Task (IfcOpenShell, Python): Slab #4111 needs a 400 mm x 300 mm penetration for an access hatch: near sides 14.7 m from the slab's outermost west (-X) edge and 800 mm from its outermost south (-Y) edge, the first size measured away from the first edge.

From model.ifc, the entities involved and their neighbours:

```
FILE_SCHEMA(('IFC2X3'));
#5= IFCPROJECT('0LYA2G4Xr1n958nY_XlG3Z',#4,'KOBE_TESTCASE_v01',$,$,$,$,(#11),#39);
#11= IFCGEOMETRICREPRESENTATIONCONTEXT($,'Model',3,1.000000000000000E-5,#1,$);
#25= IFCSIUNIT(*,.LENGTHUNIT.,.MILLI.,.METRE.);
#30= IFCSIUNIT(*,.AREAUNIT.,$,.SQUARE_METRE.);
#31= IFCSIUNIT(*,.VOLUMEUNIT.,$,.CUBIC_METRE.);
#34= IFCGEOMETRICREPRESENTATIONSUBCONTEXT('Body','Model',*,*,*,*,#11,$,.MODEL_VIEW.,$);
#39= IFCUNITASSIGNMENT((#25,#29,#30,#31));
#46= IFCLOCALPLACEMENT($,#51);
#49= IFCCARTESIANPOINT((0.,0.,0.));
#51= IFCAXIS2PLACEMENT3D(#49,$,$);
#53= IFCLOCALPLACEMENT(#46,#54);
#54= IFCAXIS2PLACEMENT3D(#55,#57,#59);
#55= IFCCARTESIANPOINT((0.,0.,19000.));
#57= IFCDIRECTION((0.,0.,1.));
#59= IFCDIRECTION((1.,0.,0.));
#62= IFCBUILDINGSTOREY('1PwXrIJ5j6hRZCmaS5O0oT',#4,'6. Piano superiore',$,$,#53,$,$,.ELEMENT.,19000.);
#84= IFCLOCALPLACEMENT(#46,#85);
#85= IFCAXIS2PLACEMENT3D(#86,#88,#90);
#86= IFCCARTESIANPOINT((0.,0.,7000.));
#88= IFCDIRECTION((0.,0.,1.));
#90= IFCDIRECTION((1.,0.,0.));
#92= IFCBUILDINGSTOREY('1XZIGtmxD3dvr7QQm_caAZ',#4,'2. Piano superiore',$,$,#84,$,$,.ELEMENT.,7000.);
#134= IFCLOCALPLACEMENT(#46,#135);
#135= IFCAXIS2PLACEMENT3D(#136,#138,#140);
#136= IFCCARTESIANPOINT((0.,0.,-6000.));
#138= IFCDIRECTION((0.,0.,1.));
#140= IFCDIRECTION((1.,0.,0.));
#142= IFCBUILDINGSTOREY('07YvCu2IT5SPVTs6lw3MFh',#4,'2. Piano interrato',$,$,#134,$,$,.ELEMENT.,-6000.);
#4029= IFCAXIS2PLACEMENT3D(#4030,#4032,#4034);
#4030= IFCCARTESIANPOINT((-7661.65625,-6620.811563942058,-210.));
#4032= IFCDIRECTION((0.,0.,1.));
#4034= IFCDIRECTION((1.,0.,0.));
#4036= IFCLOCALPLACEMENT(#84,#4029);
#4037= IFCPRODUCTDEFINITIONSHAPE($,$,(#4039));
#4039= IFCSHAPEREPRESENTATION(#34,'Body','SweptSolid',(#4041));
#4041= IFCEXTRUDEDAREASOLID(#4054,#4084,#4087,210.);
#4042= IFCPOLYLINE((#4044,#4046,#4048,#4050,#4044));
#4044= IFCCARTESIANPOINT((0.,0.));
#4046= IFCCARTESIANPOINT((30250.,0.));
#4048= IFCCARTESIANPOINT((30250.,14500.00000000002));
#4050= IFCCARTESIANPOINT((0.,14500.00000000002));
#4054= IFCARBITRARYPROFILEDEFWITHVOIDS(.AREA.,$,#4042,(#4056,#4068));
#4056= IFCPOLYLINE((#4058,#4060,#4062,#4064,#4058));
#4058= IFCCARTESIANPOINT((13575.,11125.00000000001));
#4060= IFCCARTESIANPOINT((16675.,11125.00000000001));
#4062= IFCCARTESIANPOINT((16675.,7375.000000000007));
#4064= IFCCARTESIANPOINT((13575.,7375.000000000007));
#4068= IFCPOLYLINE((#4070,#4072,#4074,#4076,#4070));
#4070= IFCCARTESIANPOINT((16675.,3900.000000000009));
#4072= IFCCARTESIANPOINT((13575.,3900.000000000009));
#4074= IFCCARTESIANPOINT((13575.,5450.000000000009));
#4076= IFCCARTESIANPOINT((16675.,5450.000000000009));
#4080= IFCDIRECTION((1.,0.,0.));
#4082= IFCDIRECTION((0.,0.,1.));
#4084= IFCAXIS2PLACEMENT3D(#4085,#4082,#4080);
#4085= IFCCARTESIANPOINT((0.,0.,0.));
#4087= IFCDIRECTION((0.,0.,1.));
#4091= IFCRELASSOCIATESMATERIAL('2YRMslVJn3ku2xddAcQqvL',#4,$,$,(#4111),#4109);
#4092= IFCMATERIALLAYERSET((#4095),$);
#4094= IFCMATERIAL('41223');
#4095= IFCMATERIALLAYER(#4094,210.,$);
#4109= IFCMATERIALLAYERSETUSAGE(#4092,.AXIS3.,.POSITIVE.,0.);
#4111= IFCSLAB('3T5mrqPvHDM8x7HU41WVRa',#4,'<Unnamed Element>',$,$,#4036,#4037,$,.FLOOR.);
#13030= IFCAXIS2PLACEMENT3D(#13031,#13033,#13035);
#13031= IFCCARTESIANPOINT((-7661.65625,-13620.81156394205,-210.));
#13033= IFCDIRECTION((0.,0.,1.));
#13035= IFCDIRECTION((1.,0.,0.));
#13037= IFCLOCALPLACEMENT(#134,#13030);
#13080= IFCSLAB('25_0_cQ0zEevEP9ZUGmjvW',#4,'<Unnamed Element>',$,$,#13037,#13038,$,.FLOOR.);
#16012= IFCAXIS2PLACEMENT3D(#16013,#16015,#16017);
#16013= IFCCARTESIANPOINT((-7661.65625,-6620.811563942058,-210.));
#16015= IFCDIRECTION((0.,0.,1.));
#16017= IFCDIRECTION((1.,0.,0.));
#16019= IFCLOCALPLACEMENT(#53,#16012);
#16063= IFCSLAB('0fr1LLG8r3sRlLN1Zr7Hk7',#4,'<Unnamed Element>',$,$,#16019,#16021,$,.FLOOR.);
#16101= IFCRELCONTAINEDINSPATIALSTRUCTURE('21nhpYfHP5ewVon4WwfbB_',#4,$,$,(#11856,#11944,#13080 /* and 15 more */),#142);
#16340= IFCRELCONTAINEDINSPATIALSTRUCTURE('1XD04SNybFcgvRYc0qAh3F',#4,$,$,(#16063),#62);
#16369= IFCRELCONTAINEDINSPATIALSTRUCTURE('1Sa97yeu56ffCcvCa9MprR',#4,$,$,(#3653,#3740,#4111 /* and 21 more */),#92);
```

```python
import numpy as np
import ifcopenshell
import ifcopenshell.api.feature
import ifcopenshell.api.geometry
import ifcopenshell.api.root
import ifcopenshell.geom
import ifcopenshell.util.placement
import ifcopenshell.util.representation
import ifcopenshell.util.shape
import ifcopenshell.util.unit

model = ifcopenshell.open("model.ifc")
unit_scale = ifcopenshell.util.unit.calculate_unit_scale(model)
settings = ifcopenshell.geom.settings()


def volume(element):
    """Net volume in cubic metres, openings subtracted."""
    shape = ifcopenshell.geom.create_shape(settings, element)
    return ifcopenshell.util.shape.get_volume(shape.geometry)


slab = model.by_guid("3T5mrqPvHDM8x7HU41WVRa")
before = volume(slab)

# Extent in the slab's own axes, in metres. The edges named are its -X and -Y sides.
slab_shape = ifcopenshell.geom.create_shape(settings, slab)
vertices = ifcopenshell.util.shape.get_vertices(slab_shape.geometry)
x_min, y_min, bottom = vertices.min(axis=0)
top = vertices[:, 2].max()

opening = ifcopenshell.api.root.create_entity(model, ifc_class="IfcOpeningElement", name="Access hatch opening")
context = ifcopenshell.util.representation.get_context(model, "Model", "Body", "MODEL_VIEW")
width, depth = 0.4, 0.3
outline = [(0.0, 0.0), (width, 0.0), (width, depth), (0.0, depth), (0.0, 0.0)]
# Overshoot both faces by 50 mm so the cut is clean.
shape = ifcopenshell.api.geometry.add_slab_representation(
    model, context=context, depth=top - bottom + 0.1, polyline=outline
)
ifcopenshell.api.geometry.assign_representation(model, product=opening, representation=shape)

matrix = ifcopenshell.util.placement.get_local_placement(slab.ObjectPlacement)
matrix[:, 3] = matrix @ np.append(np.array([x_min + 14.7, y_min + 0.8, bottom - 0.05]) / unit_scale, 1.0)
ifcopenshell.api.geometry.edit_object_placement(model, product=opening, matrix=matrix, is_si=False)
ifcopenshell.api.feature.add_feature(model, feature=opening, element=slab)

after = volume(slab)

print(f"slab volume {before:.3f} -> {after:.3f} m3")

model.write("model-out.ifc")
```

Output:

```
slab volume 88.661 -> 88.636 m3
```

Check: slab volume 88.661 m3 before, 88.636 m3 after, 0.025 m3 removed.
